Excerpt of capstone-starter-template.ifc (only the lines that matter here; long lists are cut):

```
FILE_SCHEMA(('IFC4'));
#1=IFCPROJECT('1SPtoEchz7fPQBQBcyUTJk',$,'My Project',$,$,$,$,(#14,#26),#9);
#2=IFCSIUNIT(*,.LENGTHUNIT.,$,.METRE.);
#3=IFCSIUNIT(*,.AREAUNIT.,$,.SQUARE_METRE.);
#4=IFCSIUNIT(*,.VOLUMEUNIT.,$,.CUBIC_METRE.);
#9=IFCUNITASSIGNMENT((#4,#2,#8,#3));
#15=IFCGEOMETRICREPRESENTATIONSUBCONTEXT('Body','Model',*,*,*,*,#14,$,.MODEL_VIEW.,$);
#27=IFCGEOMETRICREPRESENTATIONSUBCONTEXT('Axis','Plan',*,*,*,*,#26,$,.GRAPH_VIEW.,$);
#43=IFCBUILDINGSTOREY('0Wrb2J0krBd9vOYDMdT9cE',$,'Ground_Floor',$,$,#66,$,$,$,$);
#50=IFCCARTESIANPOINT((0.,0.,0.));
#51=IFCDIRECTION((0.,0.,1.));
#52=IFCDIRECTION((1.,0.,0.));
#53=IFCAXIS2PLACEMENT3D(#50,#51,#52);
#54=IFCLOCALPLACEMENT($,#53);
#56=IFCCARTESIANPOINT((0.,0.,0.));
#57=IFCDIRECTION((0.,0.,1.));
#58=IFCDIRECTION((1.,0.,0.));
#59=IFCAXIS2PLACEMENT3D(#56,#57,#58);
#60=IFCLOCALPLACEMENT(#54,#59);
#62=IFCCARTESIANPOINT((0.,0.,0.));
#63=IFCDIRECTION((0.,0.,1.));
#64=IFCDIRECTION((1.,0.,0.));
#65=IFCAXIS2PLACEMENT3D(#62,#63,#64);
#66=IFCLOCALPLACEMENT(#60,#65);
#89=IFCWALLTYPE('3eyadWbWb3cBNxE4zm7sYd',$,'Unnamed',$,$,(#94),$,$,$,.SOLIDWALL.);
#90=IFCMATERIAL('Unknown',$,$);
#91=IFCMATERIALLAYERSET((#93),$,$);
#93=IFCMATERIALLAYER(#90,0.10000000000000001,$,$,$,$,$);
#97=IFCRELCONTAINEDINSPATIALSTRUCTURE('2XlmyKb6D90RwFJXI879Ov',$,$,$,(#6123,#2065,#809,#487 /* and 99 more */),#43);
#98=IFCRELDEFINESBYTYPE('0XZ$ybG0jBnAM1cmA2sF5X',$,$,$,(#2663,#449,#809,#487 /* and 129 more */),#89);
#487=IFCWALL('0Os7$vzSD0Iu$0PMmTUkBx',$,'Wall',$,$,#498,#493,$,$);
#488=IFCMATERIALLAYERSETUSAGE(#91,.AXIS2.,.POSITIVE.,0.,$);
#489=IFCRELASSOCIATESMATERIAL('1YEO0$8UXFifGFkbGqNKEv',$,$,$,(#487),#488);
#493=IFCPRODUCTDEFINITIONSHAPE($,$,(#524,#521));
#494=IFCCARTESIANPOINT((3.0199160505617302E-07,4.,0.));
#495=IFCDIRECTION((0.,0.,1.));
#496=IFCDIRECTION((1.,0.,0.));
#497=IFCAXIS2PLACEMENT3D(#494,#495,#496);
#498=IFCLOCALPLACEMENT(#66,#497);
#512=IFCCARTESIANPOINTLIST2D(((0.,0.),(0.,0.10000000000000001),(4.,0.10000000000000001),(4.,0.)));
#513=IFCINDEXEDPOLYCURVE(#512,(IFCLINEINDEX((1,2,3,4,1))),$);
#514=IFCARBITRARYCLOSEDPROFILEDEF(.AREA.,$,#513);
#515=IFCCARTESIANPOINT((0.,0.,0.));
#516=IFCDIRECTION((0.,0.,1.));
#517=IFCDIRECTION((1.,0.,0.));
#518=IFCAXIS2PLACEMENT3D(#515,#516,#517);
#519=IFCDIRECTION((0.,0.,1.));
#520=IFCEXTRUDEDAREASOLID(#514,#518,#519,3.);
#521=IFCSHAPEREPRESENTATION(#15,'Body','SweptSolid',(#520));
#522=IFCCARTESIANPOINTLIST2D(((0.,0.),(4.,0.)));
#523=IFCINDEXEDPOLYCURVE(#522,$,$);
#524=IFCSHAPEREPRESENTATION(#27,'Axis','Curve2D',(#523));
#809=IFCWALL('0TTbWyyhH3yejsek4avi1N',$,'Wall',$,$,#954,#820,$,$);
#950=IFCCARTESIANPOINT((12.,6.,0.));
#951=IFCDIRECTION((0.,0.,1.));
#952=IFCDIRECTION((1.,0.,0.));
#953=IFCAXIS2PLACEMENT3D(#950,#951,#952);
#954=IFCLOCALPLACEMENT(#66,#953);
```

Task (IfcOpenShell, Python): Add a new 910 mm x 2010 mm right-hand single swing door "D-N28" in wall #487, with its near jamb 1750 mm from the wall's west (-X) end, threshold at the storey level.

```python
import numpy as np
import ifcopenshell
import ifcopenshell.api.feature
import ifcopenshell.api.geometry
import ifcopenshell.api.root
import ifcopenshell.api.spatial
import ifcopenshell.geom
import ifcopenshell.util.element
import ifcopenshell.util.placement
import ifcopenshell.util.representation
import ifcopenshell.util.shape
import ifcopenshell.util.unit

model = ifcopenshell.open("capstone-starter-template.ifc")
unit_scale = ifcopenshell.util.unit.calculate_unit_scale(model)
settings = ifcopenshell.geom.settings()


def volume(element):
    """Net volume in cubic metres, openings subtracted."""
    shape = ifcopenshell.geom.create_shape(settings, element)
    return ifcopenshell.util.shape.get_volume(shape.geometry)


wall = model.by_id(487)
storey = ifcopenshell.util.element.get_container(wall, ifc_class="IfcBuildingStorey")
context = ifcopenshell.util.representation.get_context(model, "Model", "Body", "MODEL_VIEW")
before = volume(wall)

width, height, from_end, sill = 0.91, 2.01, 1.75, 0.0  # metres

# The wall runs along its own X axis, and the end named is its -X end.
wall_shape = ifcopenshell.geom.create_shape(settings, wall)
x, y, z = ifcopenshell.util.shape.get_vertices(wall_shape.geometry).T
start = x.min() + from_end
face, thickness = float(y.min()), float(y.max() - y.min())
wall_matrix = ifcopenshell.util.placement.get_local_placement(wall.ObjectPlacement)
level = ifcopenshell.util.placement.get_local_placement(storey.ObjectPlacement)[2, 3]


def in_wall(x, y):
    """Placement at x, y metres in the wall's axes, at sill height."""
    matrix = wall_matrix.copy()
    matrix[:, 3] = wall_matrix @ np.array([x / unit_scale, y / unit_scale, 0.0, 1.0])
    matrix[2, 3] = level + sill / unit_scale
    return matrix


# Opening: a box that overshoots both wall faces by 50 mm.
opening = ifcopenshell.api.root.create_entity(model, ifc_class="IfcOpeningElement", predefined_type="OPENING")
box = ifcopenshell.api.geometry.add_wall_representation(
    model, context=context, length=width, height=height, thickness=thickness + 0.1
)
ifcopenshell.api.geometry.assign_representation(model, product=opening, representation=box)
ifcopenshell.api.geometry.edit_object_placement(model, product=opening, matrix=in_wall(start, face - 0.05), is_si=False)
ifcopenshell.api.feature.add_feature(model, feature=opening, element=wall)

door = ifcopenshell.api.root.create_entity(model, ifc_class="IfcDoor", name="D-N28", predefined_type="DOOR")
door.OverallWidth, door.OverallHeight = width / unit_scale, height / unit_scale
door.OperationType = "SINGLE_SWING_RIGHT"
body = ifcopenshell.api.geometry.add_door_representation(
    model,
    context=context,
    overall_width=door.OverallWidth,
    overall_height=door.OverallHeight,
    operation_type="SINGLE_SWING_RIGHT",
    lining_properties={"LiningDepth": thickness / unit_scale, "ThresholdDepth": thickness / unit_scale},
)
ifcopenshell.api.geometry.assign_representation(model, product=door, representation=body)
ifcopenshell.api.spatial.assign_container(model, products=[door], relating_structure=storey)
ifcopenshell.api.feature.add_filling(model, opening=opening, element=door)

# The lining spans the wall, so the door starts at the wall face.
ifcopenshell.api.geometry.edit_object_placement(model, product=door, matrix=in_wall(start, face), is_si=False)

after = volume(wall)

print(f"wall volume {before:.3f} -> {after:.3f} m3")

model.write("capstone-starter-template_v2.ifc")
```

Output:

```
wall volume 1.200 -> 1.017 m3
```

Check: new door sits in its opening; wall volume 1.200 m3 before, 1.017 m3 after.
